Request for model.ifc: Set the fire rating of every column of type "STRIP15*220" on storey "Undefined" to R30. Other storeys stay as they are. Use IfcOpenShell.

First a look at what the model holds.

```python
import ifcopenshell
import ifcopenshell.util.element

model = ifcopenshell.open("model.ifc")
print(model.schema)
storey = next(s for s in model.by_type("IfcBuildingStorey") if s.Name == "Undefined")
columns = [e for e in ifcopenshell.util.element.get_decomposition(storey) if e.is_a("IfcColumn")]
seen = {}
for e in columns:
    element_type = ifcopenshell.util.element.get_type(e)
    key = (element_type.Name if element_type != e and element_type else None, ifcopenshell.util.element.get_pset(e, "Pset_ColumnCommon", "FireRating"))
    seen[key] = seen.get(key, 0) + 1
for (name, value), count in sorted(seen.items(), key=str):
    print(count, "x", name, "|", value)
```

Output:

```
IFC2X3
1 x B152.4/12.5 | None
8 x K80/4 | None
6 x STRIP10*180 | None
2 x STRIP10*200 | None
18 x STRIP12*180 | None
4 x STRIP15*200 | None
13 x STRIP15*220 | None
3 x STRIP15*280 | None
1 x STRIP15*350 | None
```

```python
import ifcopenshell
import ifcopenshell.api.pset
import ifcopenshell.util.element

model = ifcopenshell.open("model.ifc")

storey = next(s for s in model.by_type("IfcBuildingStorey") if s.Name == "Undefined")
columns = [e for e in ifcopenshell.util.element.get_decomposition(storey) if e.is_a("IfcColumn")]

count = 0
for e in columns:
    element_type = ifcopenshell.util.element.get_type(e)
    if element_type in (None, e) or element_type.Name != "STRIP15*220":
        continue
    # add_pset returns the element's existing set when there is one.
    pset = ifcopenshell.api.pset.add_pset(model, product=e, name="Pset_ColumnCommon")
    ifcopenshell.api.pset.edit_pset(model, pset=pset, properties={"FireRating": "R30"})
    count += 1

print(count, "columns updated")

model.write("model_v2.ifc")
```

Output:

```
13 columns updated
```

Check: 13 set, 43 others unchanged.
